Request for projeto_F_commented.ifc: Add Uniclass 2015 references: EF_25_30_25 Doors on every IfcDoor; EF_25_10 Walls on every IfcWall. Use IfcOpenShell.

First a look at what the model holds.

```python
import ifcopenshell

model = ifcopenshell.open("projeto_F_commented.ifc")
print(model.schema)
print("classifications:", [c.Name for c in model.by_type("IfcClassification")])
for ifc_class in ("IfcDoor", "IfcRoof", "IfcStair", "IfcWall", "IfcWindow"):
    print(ifc_class, len(model.by_type(ifc_class)))
```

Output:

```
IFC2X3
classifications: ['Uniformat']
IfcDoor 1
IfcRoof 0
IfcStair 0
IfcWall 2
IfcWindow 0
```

```python
import ifcopenshell
import ifcopenshell.api.classification

model = ifcopenshell.open("projeto_F_commented.ifc")

# IFC2X3 requires Source and Edition and has no link from the project to the system.
system = model.create_entity("IfcClassification", Source="NBS", Edition="2015", Name="Uniclass 2015")

codes = {
    "IfcDoor": ("EF_25_30_25", "Doors"),
    "IfcWall": ("EF_25_10", "Walls"),
}
for ifc_class, (code, name) in codes.items():
    products = model.by_type(ifc_class)
    ifcopenshell.api.classification.add_reference(
        model, products=products, classification=system, identification=code, name=name
    )
    print(code, len(products))

model.write("projeto_F_commented_v2.ifc")
```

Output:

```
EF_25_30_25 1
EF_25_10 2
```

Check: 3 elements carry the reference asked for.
